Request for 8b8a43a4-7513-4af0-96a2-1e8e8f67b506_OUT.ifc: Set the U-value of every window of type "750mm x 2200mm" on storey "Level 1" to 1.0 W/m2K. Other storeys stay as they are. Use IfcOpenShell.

First a look at what the model holds.

```python
import ifcopenshell
import ifcopenshell.util.element

model = ifcopenshell.open("8b8a43a4-7513-4af0-96a2-1e8e8f67b506_OUT.ifc")
print(model.schema)
storey = next(s for s in model.by_type("IfcBuildingStorey") if s.Name == "Level 1")
windows = [e for e in ifcopenshell.util.element.get_decomposition(storey) if e.is_a("IfcWindow")]
seen = {}
for e in windows:
    element_type = ifcopenshell.util.element.get_type(e)
    key = (element_type.Name if element_type != e and element_type else None, ifcopenshell.util.element.get_pset(e, "Pset_WindowCommon", "ThermalTransmittance"))
    seen[key] = seen.get(key, 0) + 1
for (name, value), count in sorted(seen.items(), key=str):
    print(count, "x", name, "|", value)
```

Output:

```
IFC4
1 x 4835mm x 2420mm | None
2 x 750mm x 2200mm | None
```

```python
import ifcopenshell
import ifcopenshell.api.pset
import ifcopenshell.util.element

model = ifcopenshell.open("8b8a43a4-7513-4af0-96a2-1e8e8f67b506_OUT.ifc")

storey = next(s for s in model.by_type("IfcBuildingStorey") if s.Name == "Level 1")
windows = [e for e in ifcopenshell.util.element.get_decomposition(storey) if e.is_a("IfcWindow")]

count = 0
for e in windows:
    element_type = ifcopenshell.util.element.get_type(e)
    if element_type in (None, e) or element_type.Name != "750mm x 2200mm":
        continue
    # add_pset returns the element's existing set when there is one.
    pset = ifcopenshell.api.pset.add_pset(model, product=e, name="Pset_WindowCommon")
    ifcopenshell.api.pset.edit_pset(model, pset=pset, properties={"ThermalTransmittance": 1.0})
    count += 1

print(count, "windows updated")

model.write("8b8a43a4-7513-4af0-96a2-1e8e8f67b506_OUT_v2.ifc")
```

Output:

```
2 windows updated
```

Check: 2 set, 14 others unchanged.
